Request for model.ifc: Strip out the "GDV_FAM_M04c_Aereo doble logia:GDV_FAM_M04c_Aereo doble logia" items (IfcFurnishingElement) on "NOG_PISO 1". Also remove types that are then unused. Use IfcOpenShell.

First a look at what the model holds.

```python
import ifcopenshell
import ifcopenshell.util.element

model = ifcopenshell.open("model.ifc")
print(model.schema)
storey = next(s for s in model.by_type("IfcBuildingStorey") if s.Name == "NOG_PISO 1")
furniture = [e for e in ifcopenshell.util.element.get_decomposition(storey) if e.is_a("IfcFurnishingElement")]
seen = {}
for e in furniture:
    element_type = ifcopenshell.util.element.get_type(e)
    name = element_type.Name if element_type not in (None, e) else None
    seen[name] = seen.get(name, 0) + 1
for name, count in sorted(seen.items(), key=str):
    print(count, "x", name)
```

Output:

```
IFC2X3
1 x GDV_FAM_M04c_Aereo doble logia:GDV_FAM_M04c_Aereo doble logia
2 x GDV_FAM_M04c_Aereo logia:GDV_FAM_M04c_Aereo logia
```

```python
import ifcopenshell
import ifcopenshell.api.root
import ifcopenshell.util.element

model = ifcopenshell.open("model.ifc")

storey = next(s for s in model.by_type("IfcBuildingStorey") if s.Name == "NOG_PISO 1")
furniture = [e for e in ifcopenshell.util.element.get_decomposition(storey) if e.is_a("IfcFurnishingElement")]
targets = [e for e in furniture if (t := ifcopenshell.util.element.get_type(e)) not in (None, e) and t.Name == "GDV_FAM_M04c_Aereo doble logia:GDV_FAM_M04c_Aereo doble logia"]
types = {ifcopenshell.util.element.get_type(e) for e in targets} - {None, *targets}

for e in targets:
    ifcopenshell.api.root.remove_product(model, product=e)
print(len(targets), "removed")

unused = [t for t in types if not ifcopenshell.util.element.get_types(t)]
for t in unused:
    ifcopenshell.api.root.remove_product(model, product=t)
print(len(unused), "unused types removed")

model.write("model_v2.ifc")
```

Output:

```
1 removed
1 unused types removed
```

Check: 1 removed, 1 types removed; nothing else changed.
